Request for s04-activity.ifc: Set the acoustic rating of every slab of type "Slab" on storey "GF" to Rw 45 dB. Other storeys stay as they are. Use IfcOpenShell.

First a look at what the model holds.

```python
import ifcopenshell
import ifcopenshell.util.element

model = ifcopenshell.open("s04-activity.ifc")
print(model.schema)
storey = next(s for s in model.by_type("IfcBuildingStorey") if s.Name == "GF")
slabs = [e for e in ifcopenshell.util.element.get_decomposition(storey) if e.is_a("IfcSlab")]
seen = {}
for e in slabs:
    element_type = ifcopenshell.util.element.get_type(e)
    key = (element_type.Name if element_type != e and element_type else None, ifcopenshell.util.element.get_pset(e, "Pset_SlabCommon", "AcousticRating"))
    seen[key] = seen.get(key, 0) + 1
for (name, value), count in sorted(seen.items(), key=str):
    print(count, "x", name, "|", value)
```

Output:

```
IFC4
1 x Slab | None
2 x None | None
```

```python
import ifcopenshell
import ifcopenshell.api.pset
import ifcopenshell.util.element

model = ifcopenshell.open("s04-activity.ifc")

storey = next(s for s in model.by_type("IfcBuildingStorey") if s.Name == "GF")
slabs = [e for e in ifcopenshell.util.element.get_decomposition(storey) if e.is_a("IfcSlab")]

count = 0
for e in slabs:
    element_type = ifcopenshell.util.element.get_type(e)
    if element_type in (None, e) or element_type.Name != "Slab":
        continue
    # add_pset returns the element's existing set when there is one.
    pset = ifcopenshell.api.pset.add_pset(model, product=e, name="Pset_SlabCommon")
    ifcopenshell.api.pset.edit_pset(model, pset=pset, properties={"AcousticRating": "Rw 45 dB"})
    count += 1

print(count, "slabs updated")

model.write("s04-activity_rev.ifc")
```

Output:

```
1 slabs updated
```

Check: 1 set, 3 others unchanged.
